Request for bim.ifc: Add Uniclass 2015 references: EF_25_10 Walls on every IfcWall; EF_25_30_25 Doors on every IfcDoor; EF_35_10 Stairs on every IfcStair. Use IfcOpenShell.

First a look at what the model holds.

```python
import ifcopenshell

model = ifcopenshell.open("bim.ifc")
print(model.schema)
print("classifications:", [c.Name for c in model.by_type("IfcClassification")])
for ifc_class in ("IfcDoor", "IfcRoof", "IfcStair", "IfcWall", "IfcWindow"):
    print(ifc_class, len(model.by_type(ifc_class)))
```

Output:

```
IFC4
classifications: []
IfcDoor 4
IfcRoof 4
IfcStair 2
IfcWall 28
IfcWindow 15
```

```python
import ifcopenshell
import ifcopenshell.api.classification

model = ifcopenshell.open("bim.ifc")

system = ifcopenshell.api.classification.add_classification(model, classification="Uniclass 2015")

codes = {
    "IfcWall": ("EF_25_10", "Walls"),
    "IfcDoor": ("EF_25_30_25", "Doors"),
    "IfcStair": ("EF_35_10", "Stairs"),
}
for ifc_class, (code, name) in codes.items():
    products = model.by_type(ifc_class)
    ifcopenshell.api.classification.add_reference(
        model, products=products, classification=system, identification=code, name=name
    )
    print(code, len(products))

model.write("bim-out.ifc")
```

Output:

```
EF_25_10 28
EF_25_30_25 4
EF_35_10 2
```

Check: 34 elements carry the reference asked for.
